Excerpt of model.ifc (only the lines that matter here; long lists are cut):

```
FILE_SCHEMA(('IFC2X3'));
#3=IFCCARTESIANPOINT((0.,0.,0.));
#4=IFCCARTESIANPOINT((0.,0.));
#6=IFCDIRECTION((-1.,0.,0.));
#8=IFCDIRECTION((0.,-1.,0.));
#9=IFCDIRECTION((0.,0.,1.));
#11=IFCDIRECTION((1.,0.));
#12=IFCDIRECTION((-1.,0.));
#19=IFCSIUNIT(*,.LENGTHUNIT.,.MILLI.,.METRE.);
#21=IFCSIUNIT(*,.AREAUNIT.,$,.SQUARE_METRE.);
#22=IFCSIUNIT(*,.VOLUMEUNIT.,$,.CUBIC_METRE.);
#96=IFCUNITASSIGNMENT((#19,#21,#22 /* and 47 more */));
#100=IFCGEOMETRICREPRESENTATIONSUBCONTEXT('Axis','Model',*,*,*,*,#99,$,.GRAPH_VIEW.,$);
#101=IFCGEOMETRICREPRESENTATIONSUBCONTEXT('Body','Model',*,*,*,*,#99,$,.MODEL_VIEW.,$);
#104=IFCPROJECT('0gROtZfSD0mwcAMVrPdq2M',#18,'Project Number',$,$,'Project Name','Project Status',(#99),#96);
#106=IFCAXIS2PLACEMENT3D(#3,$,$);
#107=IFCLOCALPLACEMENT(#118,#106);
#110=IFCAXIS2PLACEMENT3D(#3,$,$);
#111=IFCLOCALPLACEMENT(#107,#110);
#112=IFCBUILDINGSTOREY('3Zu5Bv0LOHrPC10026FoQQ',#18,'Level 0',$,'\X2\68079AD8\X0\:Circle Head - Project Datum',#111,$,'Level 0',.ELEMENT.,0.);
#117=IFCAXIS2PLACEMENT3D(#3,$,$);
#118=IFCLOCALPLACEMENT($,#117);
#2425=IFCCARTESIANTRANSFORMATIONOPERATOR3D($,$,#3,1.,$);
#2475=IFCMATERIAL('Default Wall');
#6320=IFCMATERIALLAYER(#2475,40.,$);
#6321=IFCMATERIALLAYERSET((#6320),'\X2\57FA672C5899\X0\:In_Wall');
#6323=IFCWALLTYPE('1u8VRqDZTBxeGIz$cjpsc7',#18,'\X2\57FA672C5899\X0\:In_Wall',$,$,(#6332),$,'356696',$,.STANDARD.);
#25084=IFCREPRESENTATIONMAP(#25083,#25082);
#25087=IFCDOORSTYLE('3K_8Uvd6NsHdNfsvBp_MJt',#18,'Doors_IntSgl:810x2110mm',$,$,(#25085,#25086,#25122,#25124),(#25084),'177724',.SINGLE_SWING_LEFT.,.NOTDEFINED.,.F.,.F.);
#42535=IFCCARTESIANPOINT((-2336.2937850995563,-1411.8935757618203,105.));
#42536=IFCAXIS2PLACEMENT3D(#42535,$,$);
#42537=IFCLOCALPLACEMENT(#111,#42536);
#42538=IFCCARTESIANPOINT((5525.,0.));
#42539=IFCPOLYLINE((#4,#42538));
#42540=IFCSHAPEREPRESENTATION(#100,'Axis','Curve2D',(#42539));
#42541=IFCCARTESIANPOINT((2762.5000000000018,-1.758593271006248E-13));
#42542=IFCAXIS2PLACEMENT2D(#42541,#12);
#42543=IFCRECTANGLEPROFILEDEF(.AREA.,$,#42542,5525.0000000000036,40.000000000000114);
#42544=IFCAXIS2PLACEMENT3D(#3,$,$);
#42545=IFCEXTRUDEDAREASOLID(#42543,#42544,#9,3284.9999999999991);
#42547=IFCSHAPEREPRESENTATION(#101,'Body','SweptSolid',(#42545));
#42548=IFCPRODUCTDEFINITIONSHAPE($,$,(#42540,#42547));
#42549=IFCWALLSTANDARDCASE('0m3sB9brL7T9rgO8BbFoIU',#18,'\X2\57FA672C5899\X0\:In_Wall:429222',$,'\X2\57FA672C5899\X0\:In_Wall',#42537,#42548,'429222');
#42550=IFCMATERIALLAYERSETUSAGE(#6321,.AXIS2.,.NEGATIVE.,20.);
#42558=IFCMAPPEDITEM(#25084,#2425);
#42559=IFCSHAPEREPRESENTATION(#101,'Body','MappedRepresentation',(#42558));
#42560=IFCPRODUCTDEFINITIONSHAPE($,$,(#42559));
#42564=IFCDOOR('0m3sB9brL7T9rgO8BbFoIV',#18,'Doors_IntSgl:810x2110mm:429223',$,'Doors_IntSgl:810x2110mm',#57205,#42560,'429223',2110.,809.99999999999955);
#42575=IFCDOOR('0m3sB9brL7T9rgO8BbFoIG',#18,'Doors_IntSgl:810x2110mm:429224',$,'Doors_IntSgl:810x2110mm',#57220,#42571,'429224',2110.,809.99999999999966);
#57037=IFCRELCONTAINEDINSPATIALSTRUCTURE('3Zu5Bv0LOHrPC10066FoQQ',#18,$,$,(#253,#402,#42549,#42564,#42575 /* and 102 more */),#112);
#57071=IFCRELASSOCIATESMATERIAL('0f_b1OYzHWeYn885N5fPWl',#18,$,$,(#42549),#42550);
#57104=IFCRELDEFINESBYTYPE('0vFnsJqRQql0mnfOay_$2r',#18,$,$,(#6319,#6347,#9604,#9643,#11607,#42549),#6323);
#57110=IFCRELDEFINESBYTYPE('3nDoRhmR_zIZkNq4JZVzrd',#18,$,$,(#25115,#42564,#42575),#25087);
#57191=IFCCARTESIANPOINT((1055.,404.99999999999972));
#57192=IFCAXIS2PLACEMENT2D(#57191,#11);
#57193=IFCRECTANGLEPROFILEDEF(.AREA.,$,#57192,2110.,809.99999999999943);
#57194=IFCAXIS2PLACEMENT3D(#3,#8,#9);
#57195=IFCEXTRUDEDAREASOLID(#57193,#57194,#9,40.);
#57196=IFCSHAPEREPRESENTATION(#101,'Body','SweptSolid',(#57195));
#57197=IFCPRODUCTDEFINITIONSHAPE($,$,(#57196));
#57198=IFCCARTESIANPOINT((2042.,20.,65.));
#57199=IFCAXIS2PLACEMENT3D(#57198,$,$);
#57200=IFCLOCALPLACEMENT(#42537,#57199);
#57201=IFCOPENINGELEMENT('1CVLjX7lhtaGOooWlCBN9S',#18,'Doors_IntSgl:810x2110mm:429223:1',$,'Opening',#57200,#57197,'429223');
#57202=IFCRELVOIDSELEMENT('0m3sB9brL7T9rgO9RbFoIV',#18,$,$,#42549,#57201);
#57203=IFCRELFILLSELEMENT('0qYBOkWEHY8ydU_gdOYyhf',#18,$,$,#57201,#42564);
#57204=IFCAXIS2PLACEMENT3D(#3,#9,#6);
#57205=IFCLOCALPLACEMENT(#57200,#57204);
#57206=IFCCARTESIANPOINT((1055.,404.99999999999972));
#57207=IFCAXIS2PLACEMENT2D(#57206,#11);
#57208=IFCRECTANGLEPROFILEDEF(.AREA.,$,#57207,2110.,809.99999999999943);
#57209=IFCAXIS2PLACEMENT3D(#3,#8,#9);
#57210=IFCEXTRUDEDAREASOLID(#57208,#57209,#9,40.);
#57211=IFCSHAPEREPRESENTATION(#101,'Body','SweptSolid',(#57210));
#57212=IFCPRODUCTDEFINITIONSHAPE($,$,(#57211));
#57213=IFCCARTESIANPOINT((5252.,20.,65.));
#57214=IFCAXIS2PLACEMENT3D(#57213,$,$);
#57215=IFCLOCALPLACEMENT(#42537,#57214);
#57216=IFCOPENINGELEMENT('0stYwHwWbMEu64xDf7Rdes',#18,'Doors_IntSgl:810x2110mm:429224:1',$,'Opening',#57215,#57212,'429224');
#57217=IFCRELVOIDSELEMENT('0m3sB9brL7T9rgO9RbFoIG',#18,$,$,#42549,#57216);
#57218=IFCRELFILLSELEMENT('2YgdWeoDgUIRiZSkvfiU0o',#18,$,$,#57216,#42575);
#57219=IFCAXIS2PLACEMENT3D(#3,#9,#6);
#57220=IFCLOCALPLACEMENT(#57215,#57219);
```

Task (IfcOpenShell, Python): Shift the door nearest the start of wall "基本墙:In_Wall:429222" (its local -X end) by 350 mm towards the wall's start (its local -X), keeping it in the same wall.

```python
import ifcopenshell
import ifcopenshell.api.geometry
import ifcopenshell.util.placement
import ifcopenshell.util.unit

model = ifcopenshell.open("model.ifc")
unit_scale = ifcopenshell.util.unit.calculate_unit_scale(model)

door = model.by_guid("0m3sB9brL7T9rgO8BbFoIV")
opening = door.FillsVoids[0].RelatingOpeningElement
wall = opening.VoidsElements[0].RelatingBuildingElement

wall_matrix = ifcopenshell.util.placement.get_local_placement(wall.ObjectPlacement)
shift = wall_matrix[:3, 0] * -0.35 / unit_scale
before = ifcopenshell.util.placement.get_local_placement(door.ObjectPlacement)[:3, 3].copy()

# The door is placed relative to its opening, so it follows when the opening moves.
matrix = ifcopenshell.util.placement.get_local_placement(opening.ObjectPlacement)
matrix[:3, 3] += shift
ifcopenshell.api.geometry.edit_object_placement(
    model, product=opening, matrix=matrix, is_si=False, should_transform_children=True
)

after = ifcopenshell.util.placement.get_local_placement(door.ObjectPlacement)[:3, 3]
print("door moved by", (after - before).round(3) + 0.0)

model.write("model_edited.ifc")
```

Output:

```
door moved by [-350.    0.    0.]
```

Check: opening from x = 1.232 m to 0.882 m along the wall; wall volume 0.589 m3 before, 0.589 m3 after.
